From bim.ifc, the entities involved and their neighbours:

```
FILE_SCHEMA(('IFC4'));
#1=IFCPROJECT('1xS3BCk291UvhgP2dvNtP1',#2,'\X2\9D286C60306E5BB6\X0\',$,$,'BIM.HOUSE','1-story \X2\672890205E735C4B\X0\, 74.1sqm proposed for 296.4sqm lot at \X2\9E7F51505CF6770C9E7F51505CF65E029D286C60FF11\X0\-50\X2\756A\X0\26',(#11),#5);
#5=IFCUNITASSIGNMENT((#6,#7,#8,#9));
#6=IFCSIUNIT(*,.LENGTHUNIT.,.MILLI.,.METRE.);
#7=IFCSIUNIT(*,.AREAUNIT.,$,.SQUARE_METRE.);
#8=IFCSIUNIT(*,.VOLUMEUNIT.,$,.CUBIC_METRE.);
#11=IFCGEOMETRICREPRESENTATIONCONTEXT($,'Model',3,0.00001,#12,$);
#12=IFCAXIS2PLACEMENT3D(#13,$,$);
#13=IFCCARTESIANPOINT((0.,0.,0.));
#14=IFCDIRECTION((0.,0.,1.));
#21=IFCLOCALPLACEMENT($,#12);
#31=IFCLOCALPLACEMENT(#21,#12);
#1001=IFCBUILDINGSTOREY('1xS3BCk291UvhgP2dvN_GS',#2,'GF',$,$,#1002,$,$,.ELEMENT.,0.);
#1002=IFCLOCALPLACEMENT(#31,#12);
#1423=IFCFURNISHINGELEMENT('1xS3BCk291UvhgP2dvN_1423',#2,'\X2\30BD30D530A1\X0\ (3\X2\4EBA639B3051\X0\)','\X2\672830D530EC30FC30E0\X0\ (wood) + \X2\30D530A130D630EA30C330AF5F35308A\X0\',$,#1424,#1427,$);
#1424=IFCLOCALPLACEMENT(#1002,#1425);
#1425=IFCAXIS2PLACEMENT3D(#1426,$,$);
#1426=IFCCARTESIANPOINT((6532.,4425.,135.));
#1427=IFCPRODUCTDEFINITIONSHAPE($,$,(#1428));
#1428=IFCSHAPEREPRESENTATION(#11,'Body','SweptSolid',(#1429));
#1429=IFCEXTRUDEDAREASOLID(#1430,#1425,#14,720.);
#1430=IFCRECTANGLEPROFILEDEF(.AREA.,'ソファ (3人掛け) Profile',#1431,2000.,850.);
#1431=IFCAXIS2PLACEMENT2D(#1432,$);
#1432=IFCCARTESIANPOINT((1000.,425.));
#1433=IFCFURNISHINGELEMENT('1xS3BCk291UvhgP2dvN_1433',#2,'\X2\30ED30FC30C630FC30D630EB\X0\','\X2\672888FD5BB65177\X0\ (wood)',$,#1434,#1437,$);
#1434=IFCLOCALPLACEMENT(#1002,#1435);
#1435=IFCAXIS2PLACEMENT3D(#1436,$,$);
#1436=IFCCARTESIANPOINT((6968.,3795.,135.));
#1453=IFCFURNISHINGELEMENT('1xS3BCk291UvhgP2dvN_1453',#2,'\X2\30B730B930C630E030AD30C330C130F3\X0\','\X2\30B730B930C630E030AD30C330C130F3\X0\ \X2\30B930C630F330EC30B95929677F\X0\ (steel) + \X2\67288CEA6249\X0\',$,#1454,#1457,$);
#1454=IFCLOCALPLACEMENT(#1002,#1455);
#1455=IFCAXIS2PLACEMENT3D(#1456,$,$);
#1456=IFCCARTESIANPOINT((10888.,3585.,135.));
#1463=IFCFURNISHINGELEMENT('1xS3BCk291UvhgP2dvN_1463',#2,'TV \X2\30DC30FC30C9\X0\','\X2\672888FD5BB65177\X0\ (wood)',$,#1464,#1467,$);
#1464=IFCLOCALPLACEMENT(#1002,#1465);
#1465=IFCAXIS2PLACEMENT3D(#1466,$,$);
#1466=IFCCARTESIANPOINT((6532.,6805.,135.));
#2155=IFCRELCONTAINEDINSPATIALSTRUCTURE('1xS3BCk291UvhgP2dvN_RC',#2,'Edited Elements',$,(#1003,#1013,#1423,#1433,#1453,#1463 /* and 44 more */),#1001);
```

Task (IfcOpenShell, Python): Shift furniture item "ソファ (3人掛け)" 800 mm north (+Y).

```python
import ifcopenshell
import ifcopenshell.api.geometry
import ifcopenshell.util.placement
import ifcopenshell.util.unit

model = ifcopenshell.open("bim.ifc")
unit_scale = ifcopenshell.util.unit.calculate_unit_scale(model)

item = model.by_guid("1xS3BCk291UvhgP2dvN_1423")
matrix = ifcopenshell.util.placement.get_local_placement(item.ObjectPlacement)
matrix[1, 3] += 0.8 / unit_scale
ifcopenshell.api.geometry.edit_object_placement(model, product=item, matrix=matrix, is_si=False)

print(ifcopenshell.util.placement.get_local_placement(item.ObjectPlacement).round(3) + 0.0)

model.write("bim_updated.ifc")
```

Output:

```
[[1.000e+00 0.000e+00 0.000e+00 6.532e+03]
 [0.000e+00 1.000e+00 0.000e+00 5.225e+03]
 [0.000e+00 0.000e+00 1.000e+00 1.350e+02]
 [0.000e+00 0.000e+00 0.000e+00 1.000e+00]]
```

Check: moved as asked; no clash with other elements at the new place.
